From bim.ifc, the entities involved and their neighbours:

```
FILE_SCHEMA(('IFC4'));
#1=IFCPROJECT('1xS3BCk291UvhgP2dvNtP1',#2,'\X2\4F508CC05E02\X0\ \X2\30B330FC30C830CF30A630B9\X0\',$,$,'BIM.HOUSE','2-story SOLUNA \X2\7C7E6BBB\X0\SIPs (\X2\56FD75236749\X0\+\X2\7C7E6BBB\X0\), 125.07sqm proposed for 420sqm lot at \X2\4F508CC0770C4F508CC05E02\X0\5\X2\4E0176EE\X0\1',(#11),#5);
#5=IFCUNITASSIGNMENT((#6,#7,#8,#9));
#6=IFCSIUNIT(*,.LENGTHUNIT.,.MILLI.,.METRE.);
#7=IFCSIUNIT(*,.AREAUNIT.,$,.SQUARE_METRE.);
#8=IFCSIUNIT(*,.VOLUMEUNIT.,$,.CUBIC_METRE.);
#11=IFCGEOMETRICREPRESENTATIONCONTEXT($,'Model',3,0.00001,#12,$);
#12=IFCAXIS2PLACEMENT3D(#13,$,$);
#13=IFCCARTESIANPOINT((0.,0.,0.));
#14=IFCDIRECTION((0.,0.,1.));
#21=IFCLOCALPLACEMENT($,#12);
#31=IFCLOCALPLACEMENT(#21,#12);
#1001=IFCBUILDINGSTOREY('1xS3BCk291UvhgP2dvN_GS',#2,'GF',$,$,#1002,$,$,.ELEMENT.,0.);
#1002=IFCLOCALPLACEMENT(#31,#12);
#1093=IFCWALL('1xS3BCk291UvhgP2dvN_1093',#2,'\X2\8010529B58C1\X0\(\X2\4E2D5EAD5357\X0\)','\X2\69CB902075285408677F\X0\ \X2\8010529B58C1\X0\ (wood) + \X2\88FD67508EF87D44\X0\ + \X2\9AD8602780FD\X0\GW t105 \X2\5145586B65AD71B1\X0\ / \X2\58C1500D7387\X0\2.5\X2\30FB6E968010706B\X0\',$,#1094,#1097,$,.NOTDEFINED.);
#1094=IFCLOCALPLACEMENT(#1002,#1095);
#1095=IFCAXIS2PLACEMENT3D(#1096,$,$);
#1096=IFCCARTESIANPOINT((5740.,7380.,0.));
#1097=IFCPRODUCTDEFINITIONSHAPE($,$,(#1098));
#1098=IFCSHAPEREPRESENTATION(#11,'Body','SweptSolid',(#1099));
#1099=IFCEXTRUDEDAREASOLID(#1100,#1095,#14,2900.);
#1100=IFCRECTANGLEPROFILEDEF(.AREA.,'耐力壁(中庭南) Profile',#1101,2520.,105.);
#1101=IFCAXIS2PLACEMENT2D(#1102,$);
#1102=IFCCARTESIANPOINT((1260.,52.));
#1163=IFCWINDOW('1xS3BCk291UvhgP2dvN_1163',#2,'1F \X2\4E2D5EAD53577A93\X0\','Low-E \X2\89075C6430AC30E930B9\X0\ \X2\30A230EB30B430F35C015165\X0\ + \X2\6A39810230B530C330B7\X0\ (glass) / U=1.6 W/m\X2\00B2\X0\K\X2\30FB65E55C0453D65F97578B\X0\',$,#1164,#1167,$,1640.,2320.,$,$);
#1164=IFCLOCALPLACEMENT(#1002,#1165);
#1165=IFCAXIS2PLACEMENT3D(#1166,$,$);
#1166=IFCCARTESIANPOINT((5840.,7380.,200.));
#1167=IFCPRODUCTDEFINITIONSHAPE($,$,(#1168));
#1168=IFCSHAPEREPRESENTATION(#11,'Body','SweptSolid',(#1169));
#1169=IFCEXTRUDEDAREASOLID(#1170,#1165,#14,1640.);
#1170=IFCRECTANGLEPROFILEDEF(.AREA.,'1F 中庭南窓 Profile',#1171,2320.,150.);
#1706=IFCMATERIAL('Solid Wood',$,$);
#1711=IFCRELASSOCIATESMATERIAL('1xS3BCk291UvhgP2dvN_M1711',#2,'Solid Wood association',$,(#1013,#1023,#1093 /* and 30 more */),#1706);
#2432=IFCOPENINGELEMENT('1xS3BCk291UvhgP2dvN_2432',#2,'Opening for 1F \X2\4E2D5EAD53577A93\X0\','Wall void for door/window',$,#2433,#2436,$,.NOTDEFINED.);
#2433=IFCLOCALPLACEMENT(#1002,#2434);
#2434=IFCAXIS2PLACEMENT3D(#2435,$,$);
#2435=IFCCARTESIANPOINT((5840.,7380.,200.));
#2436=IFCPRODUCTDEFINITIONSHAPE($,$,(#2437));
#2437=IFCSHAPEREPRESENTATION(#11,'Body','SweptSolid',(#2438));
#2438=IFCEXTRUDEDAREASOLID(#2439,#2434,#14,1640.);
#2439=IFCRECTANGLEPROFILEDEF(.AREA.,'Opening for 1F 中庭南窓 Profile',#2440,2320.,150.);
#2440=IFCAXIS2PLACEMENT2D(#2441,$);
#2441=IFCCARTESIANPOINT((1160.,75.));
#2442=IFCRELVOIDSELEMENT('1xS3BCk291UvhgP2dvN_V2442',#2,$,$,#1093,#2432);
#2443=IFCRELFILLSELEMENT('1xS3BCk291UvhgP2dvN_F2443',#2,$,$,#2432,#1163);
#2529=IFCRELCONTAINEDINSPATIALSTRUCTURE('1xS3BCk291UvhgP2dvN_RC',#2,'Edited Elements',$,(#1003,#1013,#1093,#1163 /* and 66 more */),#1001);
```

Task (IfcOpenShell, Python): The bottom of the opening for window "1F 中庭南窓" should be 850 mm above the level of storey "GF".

```python
import numpy as np
import ifcopenshell
import ifcopenshell.api.geometry
import ifcopenshell.geom
import ifcopenshell.util.element
import ifcopenshell.util.placement
import ifcopenshell.util.shape
import ifcopenshell.util.unit

model = ifcopenshell.open("bim.ifc")
unit_scale = ifcopenshell.util.unit.calculate_unit_scale(model)

window = model.by_id(1163)
opening = window.FillsVoids[0].RelatingOpeningElement
storey = ifcopenshell.util.element.get_container(window, ifc_class="IfcBuildingStorey")
level = ifcopenshell.util.placement.get_local_placement(storey.ObjectPlacement)[2, 3]

# The opening's origin need not be at the sill, so measure its lowest point.
shape = ifcopenshell.geom.create_shape(ifcopenshell.geom.settings(), opening)
bottom = ifcopenshell.util.shape.get_shape_bottom_elevation(shape, shape.geometry) / unit_scale
dz = level + 850.0 - bottom

shift = np.array([0.0, 0.0, dz])
# The window is not placed relative to its opening, so move both.
for product in (opening, window):
    matrix = ifcopenshell.util.placement.get_local_placement(product.ObjectPlacement)
    matrix[:3, 3] += shift
    ifcopenshell.api.geometry.edit_object_placement(model, product=product, matrix=matrix, is_si=False)

print(f"moved by {dz * unit_scale:+.3f} m")

model.write("bim_v2.ifc")
```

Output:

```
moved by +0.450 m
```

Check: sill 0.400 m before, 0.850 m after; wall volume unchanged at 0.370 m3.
